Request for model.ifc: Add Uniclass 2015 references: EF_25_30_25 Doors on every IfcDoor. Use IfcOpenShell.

First a look at what the model holds.

```python
import ifcopenshell

model = ifcopenshell.open("model.ifc")
print(model.schema)
print("classifications:", [c.Name for c in model.by_type("IfcClassification")])
for ifc_class in ("IfcDoor", "IfcRoof", "IfcStair", "IfcWall", "IfcWindow"):
    print(ifc_class, len(model.by_type(ifc_class)))
```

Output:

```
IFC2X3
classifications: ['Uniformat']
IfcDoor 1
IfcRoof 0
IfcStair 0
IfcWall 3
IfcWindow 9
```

```python
import ifcopenshell
import ifcopenshell.api.classification

model = ifcopenshell.open("model.ifc")

# IFC2X3 requires Source and Edition and has no link from the project to the system.
system = model.create_entity("IfcClassification", Source="NBS", Edition="2015", Name="Uniclass 2015")

codes = {
    "IfcDoor": ("EF_25_30_25", "Doors"),
}
for ifc_class, (code, name) in codes.items():
    products = model.by_type(ifc_class)
    ifcopenshell.api.classification.add_reference(
        model, products=products, classification=system, identification=code, name=name
    )
    print(code, len(products))

model.write("model_rev.ifc")
```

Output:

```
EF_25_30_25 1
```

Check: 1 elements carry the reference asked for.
